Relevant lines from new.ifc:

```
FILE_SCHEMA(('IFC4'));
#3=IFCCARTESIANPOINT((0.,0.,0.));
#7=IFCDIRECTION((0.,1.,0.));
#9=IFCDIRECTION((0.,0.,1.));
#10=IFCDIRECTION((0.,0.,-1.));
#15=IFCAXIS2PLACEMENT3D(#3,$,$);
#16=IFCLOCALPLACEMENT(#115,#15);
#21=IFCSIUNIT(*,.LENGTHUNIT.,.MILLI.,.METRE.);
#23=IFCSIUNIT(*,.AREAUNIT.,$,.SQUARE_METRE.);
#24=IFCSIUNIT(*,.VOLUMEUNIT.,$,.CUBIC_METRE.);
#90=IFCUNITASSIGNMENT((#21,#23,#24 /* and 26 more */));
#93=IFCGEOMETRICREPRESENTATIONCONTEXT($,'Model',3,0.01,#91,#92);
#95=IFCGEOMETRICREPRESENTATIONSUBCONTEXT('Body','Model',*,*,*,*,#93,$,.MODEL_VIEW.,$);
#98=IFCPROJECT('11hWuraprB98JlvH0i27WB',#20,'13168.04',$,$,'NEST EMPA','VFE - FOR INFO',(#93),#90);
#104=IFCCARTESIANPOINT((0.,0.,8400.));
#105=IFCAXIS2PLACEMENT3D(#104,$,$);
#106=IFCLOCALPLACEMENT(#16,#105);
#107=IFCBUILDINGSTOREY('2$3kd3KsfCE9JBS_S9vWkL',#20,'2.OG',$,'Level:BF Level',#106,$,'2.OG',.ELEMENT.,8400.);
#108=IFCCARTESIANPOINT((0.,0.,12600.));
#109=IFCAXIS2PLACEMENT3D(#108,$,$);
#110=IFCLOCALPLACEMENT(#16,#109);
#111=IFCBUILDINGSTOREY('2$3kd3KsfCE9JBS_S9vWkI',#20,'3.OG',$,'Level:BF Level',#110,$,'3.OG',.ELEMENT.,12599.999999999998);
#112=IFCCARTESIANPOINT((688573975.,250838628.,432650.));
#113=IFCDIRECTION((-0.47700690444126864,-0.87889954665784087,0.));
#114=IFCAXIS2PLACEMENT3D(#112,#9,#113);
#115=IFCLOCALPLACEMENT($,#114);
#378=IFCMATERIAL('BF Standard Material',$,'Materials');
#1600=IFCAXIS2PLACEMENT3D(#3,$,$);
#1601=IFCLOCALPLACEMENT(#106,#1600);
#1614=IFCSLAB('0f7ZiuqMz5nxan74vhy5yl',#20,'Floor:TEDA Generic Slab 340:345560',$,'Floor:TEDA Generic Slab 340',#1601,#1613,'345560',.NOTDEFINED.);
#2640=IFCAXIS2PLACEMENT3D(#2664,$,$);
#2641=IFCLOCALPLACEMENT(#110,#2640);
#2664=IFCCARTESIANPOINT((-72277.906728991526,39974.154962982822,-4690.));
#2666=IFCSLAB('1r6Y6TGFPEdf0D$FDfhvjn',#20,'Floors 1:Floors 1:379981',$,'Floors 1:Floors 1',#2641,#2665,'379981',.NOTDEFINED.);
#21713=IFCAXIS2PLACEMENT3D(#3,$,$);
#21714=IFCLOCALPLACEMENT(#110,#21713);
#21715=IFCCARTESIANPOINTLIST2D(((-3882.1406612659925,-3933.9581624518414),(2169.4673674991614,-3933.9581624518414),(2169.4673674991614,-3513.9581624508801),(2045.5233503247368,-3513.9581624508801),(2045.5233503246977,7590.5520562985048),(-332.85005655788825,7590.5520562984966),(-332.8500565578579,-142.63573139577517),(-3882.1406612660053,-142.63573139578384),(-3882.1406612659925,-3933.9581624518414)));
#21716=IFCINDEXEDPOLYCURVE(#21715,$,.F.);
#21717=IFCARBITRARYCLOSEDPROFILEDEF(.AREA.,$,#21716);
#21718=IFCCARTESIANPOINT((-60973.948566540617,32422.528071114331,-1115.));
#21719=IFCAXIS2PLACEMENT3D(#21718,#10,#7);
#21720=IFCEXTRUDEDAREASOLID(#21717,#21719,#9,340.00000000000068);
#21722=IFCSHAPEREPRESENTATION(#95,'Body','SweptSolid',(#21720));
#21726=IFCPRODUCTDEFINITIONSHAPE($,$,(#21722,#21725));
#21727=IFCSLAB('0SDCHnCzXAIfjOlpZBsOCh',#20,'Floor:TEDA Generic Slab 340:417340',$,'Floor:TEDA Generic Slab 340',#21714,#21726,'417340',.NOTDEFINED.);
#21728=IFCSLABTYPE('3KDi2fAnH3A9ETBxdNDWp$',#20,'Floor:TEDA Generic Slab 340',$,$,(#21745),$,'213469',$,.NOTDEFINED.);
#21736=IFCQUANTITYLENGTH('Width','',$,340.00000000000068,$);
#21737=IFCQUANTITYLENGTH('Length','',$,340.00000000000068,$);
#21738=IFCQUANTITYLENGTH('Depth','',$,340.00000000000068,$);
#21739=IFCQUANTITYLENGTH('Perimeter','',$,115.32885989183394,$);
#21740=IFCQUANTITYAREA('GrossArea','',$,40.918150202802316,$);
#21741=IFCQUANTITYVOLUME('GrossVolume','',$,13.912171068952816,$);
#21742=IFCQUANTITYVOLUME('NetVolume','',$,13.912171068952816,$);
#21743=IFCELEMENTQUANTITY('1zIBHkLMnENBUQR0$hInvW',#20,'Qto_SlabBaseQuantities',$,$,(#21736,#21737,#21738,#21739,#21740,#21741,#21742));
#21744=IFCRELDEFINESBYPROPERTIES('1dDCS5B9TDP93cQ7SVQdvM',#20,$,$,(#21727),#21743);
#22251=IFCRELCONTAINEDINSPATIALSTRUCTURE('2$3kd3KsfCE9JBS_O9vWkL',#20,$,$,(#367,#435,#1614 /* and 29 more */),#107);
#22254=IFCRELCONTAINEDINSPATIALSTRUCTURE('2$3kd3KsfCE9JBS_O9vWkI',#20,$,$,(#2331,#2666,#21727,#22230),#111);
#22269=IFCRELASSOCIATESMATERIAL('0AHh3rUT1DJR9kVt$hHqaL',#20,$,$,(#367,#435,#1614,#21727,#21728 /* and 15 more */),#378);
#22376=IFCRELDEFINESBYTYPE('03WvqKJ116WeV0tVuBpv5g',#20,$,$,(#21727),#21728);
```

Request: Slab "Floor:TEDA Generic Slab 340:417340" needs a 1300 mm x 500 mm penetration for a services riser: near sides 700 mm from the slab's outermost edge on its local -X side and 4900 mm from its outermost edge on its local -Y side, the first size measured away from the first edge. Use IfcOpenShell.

```python
import numpy as np
import ifcopenshell
import ifcopenshell.api.feature
import ifcopenshell.api.geometry
import ifcopenshell.api.pset
import ifcopenshell.api.root
import ifcopenshell.geom
import ifcopenshell.util.element
import ifcopenshell.util.placement
import ifcopenshell.util.representation
import ifcopenshell.util.shape
import ifcopenshell.util.unit

model = ifcopenshell.open("new.ifc")
unit_scale = ifcopenshell.util.unit.calculate_unit_scale(model)
volume_scale = ifcopenshell.util.unit.calculate_unit_scale(model, "VOLUMEUNIT")
settings = ifcopenshell.geom.settings()


def volume(element):
    """Net volume in cubic metres, openings subtracted."""
    shape = ifcopenshell.geom.create_shape(settings, element)
    return ifcopenshell.util.shape.get_volume(shape.geometry)


slab = model.by_guid("0SDCHnCzXAIfjOlpZBsOCh")
before = volume(slab)

# Extent in the slab's own axes, in metres. The edges named are its -X and -Y sides.
slab_shape = ifcopenshell.geom.create_shape(settings, slab)
vertices = ifcopenshell.util.shape.get_vertices(slab_shape.geometry)
x_min, y_min, bottom = vertices.min(axis=0)
top = vertices[:, 2].max()

opening = ifcopenshell.api.root.create_entity(model, ifc_class="IfcOpeningElement", name="Services riser opening", predefined_type="OPENING")
context = ifcopenshell.util.representation.get_context(model, "Model", "Body", "MODEL_VIEW")
width, depth = 1.3, 0.5
outline = [(0.0, 0.0), (width, 0.0), (width, depth), (0.0, depth), (0.0, 0.0)]
# Overshoot both faces by 50 mm so the cut is clean.
shape = ifcopenshell.api.geometry.add_slab_representation(
    model, context=context, depth=top - bottom + 0.1, polyline=outline
)
ifcopenshell.api.geometry.assign_representation(model, product=opening, representation=shape)

matrix = ifcopenshell.util.placement.get_local_placement(slab.ObjectPlacement)
matrix[:, 3] = matrix @ np.append(np.array([x_min + 0.7, y_min + 4.9, bottom - 0.05]) / unit_scale, 1.0)
ifcopenshell.api.geometry.edit_object_placement(model, product=opening, matrix=matrix, is_si=False)
ifcopenshell.api.feature.add_feature(model, feature=opening, element=slab)

after = volume(slab)

# Update the slab's stored quantities.
qto = model.by_id(ifcopenshell.util.element.get_pset(slab, "Qto_SlabBaseQuantities", should_inherit=False)["id"])
ifcopenshell.api.pset.edit_qto(model, qto=qto, properties={"NetVolume": after / volume_scale})

print(f"slab volume {before:.3f} -> {after:.3f} m3")

model.write("new_updated.ifc")
```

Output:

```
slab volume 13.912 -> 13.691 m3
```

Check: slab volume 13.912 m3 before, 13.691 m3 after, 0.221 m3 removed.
